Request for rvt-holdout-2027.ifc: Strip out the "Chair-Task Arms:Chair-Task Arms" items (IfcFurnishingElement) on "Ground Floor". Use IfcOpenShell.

First a look at what the model holds.

```python
import ifcopenshell
import ifcopenshell.util.element

model = ifcopenshell.open("rvt-holdout-2027.ifc")
print(model.schema)
storey = next(s for s in model.by_type("IfcBuildingStorey") if s.Name == "Ground Floor")
furniture = [e for e in ifcopenshell.util.element.get_decomposition(storey) if e.is_a("IfcFurnishingElement")]
seen = {}
for e in furniture:
    element_type = ifcopenshell.util.element.get_type(e)
    name = element_type.Name if element_type not in (None, e) else None
    seen[name] = seen.get(name, 0) + 1
for name, count in sorted(seen.items(), key=str):
    print(count, "x", name)
```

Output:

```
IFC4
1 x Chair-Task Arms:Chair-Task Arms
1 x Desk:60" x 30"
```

```python
import ifcopenshell
import ifcopenshell.api.root
import ifcopenshell.util.element

model = ifcopenshell.open("rvt-holdout-2027.ifc")

storey = next(s for s in model.by_type("IfcBuildingStorey") if s.Name == "Ground Floor")
furniture = [e for e in ifcopenshell.util.element.get_decomposition(storey) if e.is_a("IfcFurnishingElement")]
targets = [e for e in furniture if (t := ifcopenshell.util.element.get_type(e)) not in (None, e) and t.Name == "Chair-Task Arms:Chair-Task Arms"]

for e in targets:
    ifcopenshell.api.root.remove_product(model, product=e)
print(len(targets), "removed")

model.write("rvt-holdout-2027_edited.ifc")
```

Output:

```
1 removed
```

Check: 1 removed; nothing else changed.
